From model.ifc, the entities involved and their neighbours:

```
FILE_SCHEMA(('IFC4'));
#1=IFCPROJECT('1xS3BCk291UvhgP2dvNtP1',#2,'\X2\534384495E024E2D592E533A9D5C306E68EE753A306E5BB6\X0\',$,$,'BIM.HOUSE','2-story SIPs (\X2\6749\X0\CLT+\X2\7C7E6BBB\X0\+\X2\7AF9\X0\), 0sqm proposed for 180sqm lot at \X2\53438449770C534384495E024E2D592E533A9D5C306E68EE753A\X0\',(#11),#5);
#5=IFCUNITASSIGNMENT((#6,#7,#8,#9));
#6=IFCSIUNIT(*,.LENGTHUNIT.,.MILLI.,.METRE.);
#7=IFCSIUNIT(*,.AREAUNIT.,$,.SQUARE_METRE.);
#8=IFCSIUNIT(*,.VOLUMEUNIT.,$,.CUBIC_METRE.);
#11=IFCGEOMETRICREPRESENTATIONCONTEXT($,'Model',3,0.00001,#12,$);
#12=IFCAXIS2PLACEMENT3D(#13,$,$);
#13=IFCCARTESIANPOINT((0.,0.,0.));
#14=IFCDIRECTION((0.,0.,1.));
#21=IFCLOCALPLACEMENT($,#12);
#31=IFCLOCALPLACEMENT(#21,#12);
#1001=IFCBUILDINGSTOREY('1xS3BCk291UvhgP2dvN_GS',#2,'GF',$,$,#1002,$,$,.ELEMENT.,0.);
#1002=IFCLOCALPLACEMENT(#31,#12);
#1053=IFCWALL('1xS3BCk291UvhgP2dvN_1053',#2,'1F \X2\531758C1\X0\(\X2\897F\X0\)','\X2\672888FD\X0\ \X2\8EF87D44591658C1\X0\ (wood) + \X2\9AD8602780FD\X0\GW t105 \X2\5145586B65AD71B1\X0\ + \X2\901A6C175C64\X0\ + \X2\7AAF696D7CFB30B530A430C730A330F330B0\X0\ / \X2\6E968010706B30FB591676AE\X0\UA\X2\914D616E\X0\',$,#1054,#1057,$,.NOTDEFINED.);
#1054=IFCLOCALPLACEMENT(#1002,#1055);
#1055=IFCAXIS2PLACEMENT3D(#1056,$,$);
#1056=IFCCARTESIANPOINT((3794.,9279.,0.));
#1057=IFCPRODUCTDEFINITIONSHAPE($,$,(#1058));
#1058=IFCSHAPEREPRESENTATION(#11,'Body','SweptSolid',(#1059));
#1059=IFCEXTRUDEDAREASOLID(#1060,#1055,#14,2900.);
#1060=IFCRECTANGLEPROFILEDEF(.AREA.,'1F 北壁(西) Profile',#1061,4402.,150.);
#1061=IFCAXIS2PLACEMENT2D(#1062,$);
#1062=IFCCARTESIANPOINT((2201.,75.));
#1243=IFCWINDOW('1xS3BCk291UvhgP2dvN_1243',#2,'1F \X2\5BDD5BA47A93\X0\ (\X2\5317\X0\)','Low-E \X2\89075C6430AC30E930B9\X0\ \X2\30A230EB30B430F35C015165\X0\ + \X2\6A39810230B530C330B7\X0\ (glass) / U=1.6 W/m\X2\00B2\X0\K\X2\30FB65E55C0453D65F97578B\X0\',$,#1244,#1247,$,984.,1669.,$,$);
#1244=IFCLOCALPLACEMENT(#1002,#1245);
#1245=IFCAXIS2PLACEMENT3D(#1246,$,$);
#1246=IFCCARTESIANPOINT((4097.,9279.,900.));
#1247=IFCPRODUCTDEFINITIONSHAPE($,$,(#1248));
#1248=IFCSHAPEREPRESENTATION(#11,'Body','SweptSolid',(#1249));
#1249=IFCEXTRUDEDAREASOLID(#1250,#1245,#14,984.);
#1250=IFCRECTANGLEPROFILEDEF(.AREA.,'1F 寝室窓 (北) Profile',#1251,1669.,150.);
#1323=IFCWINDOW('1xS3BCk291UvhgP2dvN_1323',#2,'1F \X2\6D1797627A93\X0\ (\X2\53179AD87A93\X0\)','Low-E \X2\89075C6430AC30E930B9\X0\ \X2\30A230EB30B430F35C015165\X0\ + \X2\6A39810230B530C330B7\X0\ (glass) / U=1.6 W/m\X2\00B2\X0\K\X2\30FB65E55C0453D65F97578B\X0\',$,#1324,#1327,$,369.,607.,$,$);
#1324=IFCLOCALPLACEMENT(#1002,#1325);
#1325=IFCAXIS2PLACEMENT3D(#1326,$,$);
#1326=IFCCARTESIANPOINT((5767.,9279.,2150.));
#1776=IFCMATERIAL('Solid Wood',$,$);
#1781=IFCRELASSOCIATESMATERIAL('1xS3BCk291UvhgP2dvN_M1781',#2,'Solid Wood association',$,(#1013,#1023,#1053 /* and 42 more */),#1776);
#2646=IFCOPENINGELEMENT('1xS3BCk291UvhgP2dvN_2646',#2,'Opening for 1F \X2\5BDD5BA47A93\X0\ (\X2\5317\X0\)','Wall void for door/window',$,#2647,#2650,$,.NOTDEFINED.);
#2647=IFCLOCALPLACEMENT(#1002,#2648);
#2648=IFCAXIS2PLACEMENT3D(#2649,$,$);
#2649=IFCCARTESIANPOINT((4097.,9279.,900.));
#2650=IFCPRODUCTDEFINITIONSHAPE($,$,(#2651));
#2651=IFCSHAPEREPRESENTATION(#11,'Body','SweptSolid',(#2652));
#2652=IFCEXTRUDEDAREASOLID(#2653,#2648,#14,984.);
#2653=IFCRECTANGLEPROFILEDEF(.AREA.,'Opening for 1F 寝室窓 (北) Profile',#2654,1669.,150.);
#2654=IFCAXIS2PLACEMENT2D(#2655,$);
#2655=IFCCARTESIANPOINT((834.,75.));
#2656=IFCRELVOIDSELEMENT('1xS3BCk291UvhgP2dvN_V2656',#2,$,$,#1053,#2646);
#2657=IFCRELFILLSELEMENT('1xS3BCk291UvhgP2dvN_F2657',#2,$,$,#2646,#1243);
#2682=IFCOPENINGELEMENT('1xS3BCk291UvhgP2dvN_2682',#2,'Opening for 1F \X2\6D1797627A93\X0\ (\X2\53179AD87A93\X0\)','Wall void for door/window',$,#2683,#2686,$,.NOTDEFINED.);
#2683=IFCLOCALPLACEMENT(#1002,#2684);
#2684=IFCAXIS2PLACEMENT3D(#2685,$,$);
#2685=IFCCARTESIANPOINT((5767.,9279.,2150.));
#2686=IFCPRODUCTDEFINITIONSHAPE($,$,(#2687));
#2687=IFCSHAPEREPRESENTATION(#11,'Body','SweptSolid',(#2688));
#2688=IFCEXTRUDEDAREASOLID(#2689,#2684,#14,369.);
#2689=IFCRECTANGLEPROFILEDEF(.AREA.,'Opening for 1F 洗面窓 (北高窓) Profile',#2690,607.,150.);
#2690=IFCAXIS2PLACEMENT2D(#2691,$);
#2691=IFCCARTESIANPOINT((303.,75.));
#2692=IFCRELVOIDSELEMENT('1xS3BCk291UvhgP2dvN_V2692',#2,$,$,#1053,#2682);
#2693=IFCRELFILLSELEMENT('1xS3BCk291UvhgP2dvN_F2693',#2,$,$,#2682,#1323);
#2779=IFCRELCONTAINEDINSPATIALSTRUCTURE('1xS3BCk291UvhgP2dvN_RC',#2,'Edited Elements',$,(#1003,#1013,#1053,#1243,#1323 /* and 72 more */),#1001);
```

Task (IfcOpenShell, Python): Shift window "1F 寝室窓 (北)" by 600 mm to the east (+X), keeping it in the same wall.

```python
import ifcopenshell
import ifcopenshell.api.geometry
import ifcopenshell.util.placement
import ifcopenshell.util.unit

model = ifcopenshell.open("model.ifc")
unit_scale = ifcopenshell.util.unit.calculate_unit_scale(model)

window = model.by_guid("1xS3BCk291UvhgP2dvN_1243")
opening = window.FillsVoids[0].RelatingOpeningElement
wall = opening.VoidsElements[0].RelatingBuildingElement

wall_matrix = ifcopenshell.util.placement.get_local_placement(wall.ObjectPlacement)
shift = wall_matrix[:3, 0] * 0.6 / unit_scale
before = ifcopenshell.util.placement.get_local_placement(window.ObjectPlacement)[:3, 3].copy()

# The window is not placed relative to its opening, so move both.
for product in (opening, window):
    matrix = ifcopenshell.util.placement.get_local_placement(product.ObjectPlacement)
    matrix[:3, 3] += shift
    ifcopenshell.api.geometry.edit_object_placement(model, product=product, matrix=matrix, is_si=False)

after = ifcopenshell.util.placement.get_local_placement(window.ObjectPlacement)[:3, 3]
print("window moved by", (after - before).round(3) + 0.0)

model.write("model_updated.ifc")
```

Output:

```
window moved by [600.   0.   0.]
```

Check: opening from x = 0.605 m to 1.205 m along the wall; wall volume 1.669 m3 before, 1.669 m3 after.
